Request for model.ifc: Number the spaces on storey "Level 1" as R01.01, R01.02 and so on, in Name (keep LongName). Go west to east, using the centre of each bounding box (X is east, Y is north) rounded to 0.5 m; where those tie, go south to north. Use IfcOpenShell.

First a look at what the model holds.

```python
import ifcopenshell
import ifcopenshell.util.element
import ifcopenshell.util.placement

model = ifcopenshell.open("model.ifc")
print(model.schema)
storey = next(s for s in model.by_type("IfcBuildingStorey") if s.Name == "Level 1")
spaces = [e for e in ifcopenshell.util.element.get_decomposition(storey) if e.is_a("IfcSpace")]
for e in sorted(spaces, key=lambda e: e.id()):
    origin = ifcopenshell.util.placement.get_local_placement(e.ObjectPlacement)[:3, 3]
    print(e.id(), e.Name, e.LongName, origin.round(2) + 0.0, sep=" | ")
```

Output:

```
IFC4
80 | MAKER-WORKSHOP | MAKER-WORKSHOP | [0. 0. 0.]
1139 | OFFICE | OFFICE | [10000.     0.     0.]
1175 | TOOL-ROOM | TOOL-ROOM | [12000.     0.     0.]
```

```python
import ifcopenshell
import ifcopenshell.geom
import ifcopenshell.util.element
import ifcopenshell.util.shape

model = ifcopenshell.open("model.ifc")
settings = ifcopenshell.geom.settings()
settings.set("use-world-coords", True)


def centre(element):
    shape = ifcopenshell.geom.create_shape(settings, element)
    return ifcopenshell.util.shape.get_bbox_centroid(shape.geometry)


storey = next(s for s in model.by_type("IfcBuildingStorey") if s.Name == "Level 1")
spaces = [e for e in ifcopenshell.util.element.get_decomposition(storey) if e.is_a("IfcSpace")]

# Insertion points can sit at a corner or the storey origin, so sort by the geometry (in metres).
centres = {e: centre(e) for e in spaces}
spaces.sort(key=lambda e: (round(centres[e][0] / 0.5), centres[e][1]))

for i, e in enumerate(spaces, start=1):
    number = f"R01.{i:02d}"
    e.Name = number
    print(e.id(), number)

model.write("model_rev.ifc")
```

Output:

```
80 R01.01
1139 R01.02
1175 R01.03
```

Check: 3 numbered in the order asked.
